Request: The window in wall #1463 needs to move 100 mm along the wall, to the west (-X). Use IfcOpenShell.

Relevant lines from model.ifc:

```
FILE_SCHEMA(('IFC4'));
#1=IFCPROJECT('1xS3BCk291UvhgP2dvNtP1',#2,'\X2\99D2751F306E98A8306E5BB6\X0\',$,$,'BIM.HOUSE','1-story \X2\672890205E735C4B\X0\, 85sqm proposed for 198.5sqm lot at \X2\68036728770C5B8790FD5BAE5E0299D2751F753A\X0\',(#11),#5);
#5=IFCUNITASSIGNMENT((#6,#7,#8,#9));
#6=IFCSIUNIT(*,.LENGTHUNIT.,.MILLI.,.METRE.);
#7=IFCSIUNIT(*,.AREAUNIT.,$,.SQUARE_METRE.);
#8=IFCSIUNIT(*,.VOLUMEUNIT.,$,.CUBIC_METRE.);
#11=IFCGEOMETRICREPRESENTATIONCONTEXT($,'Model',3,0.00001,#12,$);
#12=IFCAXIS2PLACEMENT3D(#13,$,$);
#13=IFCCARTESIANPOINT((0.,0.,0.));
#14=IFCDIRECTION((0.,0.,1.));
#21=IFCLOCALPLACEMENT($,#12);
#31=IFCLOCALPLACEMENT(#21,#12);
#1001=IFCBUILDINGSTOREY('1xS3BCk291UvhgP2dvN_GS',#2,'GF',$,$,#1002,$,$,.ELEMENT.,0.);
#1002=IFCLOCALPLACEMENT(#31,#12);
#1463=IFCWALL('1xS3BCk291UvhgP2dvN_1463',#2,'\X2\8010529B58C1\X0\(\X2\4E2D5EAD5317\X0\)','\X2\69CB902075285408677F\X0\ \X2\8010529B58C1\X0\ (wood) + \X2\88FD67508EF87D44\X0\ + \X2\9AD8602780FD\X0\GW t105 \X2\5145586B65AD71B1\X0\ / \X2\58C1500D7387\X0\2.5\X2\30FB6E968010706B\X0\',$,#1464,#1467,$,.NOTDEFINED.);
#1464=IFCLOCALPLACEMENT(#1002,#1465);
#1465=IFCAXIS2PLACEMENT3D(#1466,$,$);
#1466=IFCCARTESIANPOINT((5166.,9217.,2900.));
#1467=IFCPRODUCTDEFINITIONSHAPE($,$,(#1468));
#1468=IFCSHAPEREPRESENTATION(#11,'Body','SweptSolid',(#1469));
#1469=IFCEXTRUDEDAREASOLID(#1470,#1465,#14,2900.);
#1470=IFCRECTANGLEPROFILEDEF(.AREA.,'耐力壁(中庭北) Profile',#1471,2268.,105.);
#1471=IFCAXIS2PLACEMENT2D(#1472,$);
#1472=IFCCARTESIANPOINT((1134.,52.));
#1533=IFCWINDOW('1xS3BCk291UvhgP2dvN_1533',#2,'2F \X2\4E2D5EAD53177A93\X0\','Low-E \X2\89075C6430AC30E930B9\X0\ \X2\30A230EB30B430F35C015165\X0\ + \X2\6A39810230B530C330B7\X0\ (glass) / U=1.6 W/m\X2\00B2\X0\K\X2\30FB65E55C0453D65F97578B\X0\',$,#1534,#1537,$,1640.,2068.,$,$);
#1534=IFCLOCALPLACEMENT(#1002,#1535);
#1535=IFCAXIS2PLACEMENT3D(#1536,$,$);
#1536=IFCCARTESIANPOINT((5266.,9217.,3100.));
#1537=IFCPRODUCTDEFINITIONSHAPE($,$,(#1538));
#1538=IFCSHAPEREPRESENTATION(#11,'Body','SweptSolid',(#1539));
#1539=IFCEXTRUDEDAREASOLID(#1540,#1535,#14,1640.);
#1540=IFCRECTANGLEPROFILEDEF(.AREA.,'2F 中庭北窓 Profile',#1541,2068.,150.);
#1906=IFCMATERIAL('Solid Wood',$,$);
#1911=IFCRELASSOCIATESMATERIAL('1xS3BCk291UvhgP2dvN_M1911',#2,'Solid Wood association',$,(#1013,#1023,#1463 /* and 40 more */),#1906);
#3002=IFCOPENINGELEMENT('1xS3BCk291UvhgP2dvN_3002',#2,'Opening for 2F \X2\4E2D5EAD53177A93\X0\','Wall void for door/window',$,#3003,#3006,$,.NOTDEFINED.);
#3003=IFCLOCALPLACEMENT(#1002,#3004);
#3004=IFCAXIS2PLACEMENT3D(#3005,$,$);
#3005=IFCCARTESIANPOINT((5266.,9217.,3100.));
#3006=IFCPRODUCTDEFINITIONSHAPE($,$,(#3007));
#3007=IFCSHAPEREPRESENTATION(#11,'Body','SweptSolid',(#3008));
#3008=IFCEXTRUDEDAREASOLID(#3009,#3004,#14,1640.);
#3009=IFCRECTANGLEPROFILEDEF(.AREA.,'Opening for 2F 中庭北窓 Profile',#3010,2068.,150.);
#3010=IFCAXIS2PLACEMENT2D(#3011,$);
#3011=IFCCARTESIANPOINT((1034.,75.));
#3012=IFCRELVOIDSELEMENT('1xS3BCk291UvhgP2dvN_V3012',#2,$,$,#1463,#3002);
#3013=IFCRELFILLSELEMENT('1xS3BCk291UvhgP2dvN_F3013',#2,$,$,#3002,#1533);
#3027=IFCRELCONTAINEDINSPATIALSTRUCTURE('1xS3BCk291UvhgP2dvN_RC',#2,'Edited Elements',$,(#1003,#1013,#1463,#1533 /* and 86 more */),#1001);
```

```python
import ifcopenshell
import ifcopenshell.api.geometry
import ifcopenshell.util.placement

model = ifcopenshell.open("model.ifc")

window = model.by_id(1533)
opening = window.FillsVoids[0].RelatingOpeningElement
wall = opening.VoidsElements[0].RelatingBuildingElement

wall_matrix = ifcopenshell.util.placement.get_local_placement(wall.ObjectPlacement)
shift = wall_matrix[:3, 0] * -100.0
before = ifcopenshell.util.placement.get_local_placement(window.ObjectPlacement)[:3, 3].copy()

# The window is not placed relative to its opening, so move both.
for product in (opening, window):
    matrix = ifcopenshell.util.placement.get_local_placement(product.ObjectPlacement)
    matrix[:3, 3] += shift
    ifcopenshell.api.geometry.edit_object_placement(model, product=product, matrix=matrix, is_si=False)

after = ifcopenshell.util.placement.get_local_placement(window.ObjectPlacement)[:3, 3]
print("window moved by", (after - before).round(3) + 0.0)

model.write("model-out.ifc")
```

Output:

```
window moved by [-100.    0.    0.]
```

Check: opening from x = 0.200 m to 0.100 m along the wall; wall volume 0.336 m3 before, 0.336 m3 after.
